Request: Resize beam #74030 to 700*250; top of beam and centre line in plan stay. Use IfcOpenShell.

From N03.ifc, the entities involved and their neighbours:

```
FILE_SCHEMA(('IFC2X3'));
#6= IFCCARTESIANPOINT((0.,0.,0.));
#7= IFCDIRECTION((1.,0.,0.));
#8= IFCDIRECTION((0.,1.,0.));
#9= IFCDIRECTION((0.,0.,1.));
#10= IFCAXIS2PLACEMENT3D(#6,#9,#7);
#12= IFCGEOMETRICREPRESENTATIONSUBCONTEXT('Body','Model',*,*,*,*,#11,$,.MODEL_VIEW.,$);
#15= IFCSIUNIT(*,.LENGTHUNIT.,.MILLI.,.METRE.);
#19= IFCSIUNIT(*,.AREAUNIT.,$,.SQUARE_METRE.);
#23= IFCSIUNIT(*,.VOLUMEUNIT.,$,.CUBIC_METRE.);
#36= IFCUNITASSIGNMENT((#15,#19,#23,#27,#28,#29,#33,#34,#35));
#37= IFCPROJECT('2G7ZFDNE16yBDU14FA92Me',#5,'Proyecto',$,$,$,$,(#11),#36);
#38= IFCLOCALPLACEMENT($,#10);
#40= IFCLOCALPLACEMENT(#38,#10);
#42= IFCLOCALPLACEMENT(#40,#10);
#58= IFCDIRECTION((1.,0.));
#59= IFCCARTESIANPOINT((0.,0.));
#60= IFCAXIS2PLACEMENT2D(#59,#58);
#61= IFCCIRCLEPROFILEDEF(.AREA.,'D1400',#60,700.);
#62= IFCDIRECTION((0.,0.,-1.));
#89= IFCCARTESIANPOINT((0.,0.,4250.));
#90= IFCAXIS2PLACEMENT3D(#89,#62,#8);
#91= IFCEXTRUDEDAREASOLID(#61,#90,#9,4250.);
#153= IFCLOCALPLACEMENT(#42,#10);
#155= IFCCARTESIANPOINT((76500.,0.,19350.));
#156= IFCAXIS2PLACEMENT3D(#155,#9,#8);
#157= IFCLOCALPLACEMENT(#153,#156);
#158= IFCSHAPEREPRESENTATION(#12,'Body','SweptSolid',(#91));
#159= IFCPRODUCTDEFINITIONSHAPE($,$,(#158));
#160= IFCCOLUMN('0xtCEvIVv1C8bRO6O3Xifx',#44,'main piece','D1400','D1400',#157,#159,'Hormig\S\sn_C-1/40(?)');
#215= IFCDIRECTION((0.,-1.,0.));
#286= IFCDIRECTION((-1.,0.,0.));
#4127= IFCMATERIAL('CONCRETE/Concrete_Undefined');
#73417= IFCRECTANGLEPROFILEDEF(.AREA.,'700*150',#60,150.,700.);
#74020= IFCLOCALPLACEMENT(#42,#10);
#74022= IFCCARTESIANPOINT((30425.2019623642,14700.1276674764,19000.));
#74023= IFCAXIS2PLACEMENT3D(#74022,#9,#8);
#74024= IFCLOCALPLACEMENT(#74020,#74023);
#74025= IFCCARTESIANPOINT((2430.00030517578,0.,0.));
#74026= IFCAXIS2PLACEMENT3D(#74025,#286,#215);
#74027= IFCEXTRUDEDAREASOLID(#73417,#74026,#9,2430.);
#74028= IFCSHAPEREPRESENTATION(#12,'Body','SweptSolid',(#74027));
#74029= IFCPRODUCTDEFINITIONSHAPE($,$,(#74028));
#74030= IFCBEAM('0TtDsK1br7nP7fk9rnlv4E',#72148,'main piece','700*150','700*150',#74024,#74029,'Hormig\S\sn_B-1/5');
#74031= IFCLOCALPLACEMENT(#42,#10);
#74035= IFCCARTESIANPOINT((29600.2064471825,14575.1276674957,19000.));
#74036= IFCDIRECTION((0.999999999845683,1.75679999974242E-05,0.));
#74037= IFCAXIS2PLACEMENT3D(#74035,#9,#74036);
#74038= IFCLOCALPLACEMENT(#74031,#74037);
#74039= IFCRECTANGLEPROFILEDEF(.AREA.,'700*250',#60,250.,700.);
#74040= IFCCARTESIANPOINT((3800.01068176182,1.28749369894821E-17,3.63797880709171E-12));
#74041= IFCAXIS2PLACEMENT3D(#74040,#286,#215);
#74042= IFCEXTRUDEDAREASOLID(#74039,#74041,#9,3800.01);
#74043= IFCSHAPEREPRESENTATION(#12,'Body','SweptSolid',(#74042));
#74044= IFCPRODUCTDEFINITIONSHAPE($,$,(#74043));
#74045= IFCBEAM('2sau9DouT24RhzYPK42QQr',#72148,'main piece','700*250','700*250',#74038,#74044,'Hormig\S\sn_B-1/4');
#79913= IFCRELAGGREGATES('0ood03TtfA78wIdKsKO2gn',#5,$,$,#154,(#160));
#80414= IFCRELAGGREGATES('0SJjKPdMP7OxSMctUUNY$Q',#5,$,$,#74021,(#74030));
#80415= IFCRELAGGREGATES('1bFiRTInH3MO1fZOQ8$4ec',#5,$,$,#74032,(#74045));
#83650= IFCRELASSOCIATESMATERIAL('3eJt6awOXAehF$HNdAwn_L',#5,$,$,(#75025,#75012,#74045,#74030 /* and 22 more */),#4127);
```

```python
import ifcopenshell
import ifcopenshell.util.element
import ifcopenshell.util.representation

model = ifcopenshell.open("N03.ifc")

member = model.by_id(74030)
source = next(p for p in model.by_type("IfcRectangleProfileDef") if p.ProfileName == "700*250")

body = ifcopenshell.util.representation.get_representation(member, "Model", "Body")
solid = body.Items[0]
old_profile = solid.SweptArea

# Copy the section's sizes but keep this member's own profile position.
profile = ifcopenshell.util.element.copy(model, source)
# Profiles are centred, so shift by half the change in depth to hold the top.
shift = (old_profile.YDim - profile.YDim) / 2
x, y = old_profile.Position.Location.Coordinates
up = (0.0, 1.0)  # upwards, in the solid's own plane
location = model.createIfcCartesianPoint((x + up[0] * shift, y + up[1] * shift))
profile.Position = model.createIfcAxis2Placement2D(location, old_profile.Position.RefDirection)
solid.SweptArea = profile
if not model.get_total_inverses(old_profile):
    ifcopenshell.util.element.remove_deep2(model, old_profile)
member.Description = member.Description.replace("700*150", "700*250")
member.ObjectType = member.ObjectType.replace("700*150", "700*250")

print(solid.SweptArea)

model.write("N03_rev.ifc")
```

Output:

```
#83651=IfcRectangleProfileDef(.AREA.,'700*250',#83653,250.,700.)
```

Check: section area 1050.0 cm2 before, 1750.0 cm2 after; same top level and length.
